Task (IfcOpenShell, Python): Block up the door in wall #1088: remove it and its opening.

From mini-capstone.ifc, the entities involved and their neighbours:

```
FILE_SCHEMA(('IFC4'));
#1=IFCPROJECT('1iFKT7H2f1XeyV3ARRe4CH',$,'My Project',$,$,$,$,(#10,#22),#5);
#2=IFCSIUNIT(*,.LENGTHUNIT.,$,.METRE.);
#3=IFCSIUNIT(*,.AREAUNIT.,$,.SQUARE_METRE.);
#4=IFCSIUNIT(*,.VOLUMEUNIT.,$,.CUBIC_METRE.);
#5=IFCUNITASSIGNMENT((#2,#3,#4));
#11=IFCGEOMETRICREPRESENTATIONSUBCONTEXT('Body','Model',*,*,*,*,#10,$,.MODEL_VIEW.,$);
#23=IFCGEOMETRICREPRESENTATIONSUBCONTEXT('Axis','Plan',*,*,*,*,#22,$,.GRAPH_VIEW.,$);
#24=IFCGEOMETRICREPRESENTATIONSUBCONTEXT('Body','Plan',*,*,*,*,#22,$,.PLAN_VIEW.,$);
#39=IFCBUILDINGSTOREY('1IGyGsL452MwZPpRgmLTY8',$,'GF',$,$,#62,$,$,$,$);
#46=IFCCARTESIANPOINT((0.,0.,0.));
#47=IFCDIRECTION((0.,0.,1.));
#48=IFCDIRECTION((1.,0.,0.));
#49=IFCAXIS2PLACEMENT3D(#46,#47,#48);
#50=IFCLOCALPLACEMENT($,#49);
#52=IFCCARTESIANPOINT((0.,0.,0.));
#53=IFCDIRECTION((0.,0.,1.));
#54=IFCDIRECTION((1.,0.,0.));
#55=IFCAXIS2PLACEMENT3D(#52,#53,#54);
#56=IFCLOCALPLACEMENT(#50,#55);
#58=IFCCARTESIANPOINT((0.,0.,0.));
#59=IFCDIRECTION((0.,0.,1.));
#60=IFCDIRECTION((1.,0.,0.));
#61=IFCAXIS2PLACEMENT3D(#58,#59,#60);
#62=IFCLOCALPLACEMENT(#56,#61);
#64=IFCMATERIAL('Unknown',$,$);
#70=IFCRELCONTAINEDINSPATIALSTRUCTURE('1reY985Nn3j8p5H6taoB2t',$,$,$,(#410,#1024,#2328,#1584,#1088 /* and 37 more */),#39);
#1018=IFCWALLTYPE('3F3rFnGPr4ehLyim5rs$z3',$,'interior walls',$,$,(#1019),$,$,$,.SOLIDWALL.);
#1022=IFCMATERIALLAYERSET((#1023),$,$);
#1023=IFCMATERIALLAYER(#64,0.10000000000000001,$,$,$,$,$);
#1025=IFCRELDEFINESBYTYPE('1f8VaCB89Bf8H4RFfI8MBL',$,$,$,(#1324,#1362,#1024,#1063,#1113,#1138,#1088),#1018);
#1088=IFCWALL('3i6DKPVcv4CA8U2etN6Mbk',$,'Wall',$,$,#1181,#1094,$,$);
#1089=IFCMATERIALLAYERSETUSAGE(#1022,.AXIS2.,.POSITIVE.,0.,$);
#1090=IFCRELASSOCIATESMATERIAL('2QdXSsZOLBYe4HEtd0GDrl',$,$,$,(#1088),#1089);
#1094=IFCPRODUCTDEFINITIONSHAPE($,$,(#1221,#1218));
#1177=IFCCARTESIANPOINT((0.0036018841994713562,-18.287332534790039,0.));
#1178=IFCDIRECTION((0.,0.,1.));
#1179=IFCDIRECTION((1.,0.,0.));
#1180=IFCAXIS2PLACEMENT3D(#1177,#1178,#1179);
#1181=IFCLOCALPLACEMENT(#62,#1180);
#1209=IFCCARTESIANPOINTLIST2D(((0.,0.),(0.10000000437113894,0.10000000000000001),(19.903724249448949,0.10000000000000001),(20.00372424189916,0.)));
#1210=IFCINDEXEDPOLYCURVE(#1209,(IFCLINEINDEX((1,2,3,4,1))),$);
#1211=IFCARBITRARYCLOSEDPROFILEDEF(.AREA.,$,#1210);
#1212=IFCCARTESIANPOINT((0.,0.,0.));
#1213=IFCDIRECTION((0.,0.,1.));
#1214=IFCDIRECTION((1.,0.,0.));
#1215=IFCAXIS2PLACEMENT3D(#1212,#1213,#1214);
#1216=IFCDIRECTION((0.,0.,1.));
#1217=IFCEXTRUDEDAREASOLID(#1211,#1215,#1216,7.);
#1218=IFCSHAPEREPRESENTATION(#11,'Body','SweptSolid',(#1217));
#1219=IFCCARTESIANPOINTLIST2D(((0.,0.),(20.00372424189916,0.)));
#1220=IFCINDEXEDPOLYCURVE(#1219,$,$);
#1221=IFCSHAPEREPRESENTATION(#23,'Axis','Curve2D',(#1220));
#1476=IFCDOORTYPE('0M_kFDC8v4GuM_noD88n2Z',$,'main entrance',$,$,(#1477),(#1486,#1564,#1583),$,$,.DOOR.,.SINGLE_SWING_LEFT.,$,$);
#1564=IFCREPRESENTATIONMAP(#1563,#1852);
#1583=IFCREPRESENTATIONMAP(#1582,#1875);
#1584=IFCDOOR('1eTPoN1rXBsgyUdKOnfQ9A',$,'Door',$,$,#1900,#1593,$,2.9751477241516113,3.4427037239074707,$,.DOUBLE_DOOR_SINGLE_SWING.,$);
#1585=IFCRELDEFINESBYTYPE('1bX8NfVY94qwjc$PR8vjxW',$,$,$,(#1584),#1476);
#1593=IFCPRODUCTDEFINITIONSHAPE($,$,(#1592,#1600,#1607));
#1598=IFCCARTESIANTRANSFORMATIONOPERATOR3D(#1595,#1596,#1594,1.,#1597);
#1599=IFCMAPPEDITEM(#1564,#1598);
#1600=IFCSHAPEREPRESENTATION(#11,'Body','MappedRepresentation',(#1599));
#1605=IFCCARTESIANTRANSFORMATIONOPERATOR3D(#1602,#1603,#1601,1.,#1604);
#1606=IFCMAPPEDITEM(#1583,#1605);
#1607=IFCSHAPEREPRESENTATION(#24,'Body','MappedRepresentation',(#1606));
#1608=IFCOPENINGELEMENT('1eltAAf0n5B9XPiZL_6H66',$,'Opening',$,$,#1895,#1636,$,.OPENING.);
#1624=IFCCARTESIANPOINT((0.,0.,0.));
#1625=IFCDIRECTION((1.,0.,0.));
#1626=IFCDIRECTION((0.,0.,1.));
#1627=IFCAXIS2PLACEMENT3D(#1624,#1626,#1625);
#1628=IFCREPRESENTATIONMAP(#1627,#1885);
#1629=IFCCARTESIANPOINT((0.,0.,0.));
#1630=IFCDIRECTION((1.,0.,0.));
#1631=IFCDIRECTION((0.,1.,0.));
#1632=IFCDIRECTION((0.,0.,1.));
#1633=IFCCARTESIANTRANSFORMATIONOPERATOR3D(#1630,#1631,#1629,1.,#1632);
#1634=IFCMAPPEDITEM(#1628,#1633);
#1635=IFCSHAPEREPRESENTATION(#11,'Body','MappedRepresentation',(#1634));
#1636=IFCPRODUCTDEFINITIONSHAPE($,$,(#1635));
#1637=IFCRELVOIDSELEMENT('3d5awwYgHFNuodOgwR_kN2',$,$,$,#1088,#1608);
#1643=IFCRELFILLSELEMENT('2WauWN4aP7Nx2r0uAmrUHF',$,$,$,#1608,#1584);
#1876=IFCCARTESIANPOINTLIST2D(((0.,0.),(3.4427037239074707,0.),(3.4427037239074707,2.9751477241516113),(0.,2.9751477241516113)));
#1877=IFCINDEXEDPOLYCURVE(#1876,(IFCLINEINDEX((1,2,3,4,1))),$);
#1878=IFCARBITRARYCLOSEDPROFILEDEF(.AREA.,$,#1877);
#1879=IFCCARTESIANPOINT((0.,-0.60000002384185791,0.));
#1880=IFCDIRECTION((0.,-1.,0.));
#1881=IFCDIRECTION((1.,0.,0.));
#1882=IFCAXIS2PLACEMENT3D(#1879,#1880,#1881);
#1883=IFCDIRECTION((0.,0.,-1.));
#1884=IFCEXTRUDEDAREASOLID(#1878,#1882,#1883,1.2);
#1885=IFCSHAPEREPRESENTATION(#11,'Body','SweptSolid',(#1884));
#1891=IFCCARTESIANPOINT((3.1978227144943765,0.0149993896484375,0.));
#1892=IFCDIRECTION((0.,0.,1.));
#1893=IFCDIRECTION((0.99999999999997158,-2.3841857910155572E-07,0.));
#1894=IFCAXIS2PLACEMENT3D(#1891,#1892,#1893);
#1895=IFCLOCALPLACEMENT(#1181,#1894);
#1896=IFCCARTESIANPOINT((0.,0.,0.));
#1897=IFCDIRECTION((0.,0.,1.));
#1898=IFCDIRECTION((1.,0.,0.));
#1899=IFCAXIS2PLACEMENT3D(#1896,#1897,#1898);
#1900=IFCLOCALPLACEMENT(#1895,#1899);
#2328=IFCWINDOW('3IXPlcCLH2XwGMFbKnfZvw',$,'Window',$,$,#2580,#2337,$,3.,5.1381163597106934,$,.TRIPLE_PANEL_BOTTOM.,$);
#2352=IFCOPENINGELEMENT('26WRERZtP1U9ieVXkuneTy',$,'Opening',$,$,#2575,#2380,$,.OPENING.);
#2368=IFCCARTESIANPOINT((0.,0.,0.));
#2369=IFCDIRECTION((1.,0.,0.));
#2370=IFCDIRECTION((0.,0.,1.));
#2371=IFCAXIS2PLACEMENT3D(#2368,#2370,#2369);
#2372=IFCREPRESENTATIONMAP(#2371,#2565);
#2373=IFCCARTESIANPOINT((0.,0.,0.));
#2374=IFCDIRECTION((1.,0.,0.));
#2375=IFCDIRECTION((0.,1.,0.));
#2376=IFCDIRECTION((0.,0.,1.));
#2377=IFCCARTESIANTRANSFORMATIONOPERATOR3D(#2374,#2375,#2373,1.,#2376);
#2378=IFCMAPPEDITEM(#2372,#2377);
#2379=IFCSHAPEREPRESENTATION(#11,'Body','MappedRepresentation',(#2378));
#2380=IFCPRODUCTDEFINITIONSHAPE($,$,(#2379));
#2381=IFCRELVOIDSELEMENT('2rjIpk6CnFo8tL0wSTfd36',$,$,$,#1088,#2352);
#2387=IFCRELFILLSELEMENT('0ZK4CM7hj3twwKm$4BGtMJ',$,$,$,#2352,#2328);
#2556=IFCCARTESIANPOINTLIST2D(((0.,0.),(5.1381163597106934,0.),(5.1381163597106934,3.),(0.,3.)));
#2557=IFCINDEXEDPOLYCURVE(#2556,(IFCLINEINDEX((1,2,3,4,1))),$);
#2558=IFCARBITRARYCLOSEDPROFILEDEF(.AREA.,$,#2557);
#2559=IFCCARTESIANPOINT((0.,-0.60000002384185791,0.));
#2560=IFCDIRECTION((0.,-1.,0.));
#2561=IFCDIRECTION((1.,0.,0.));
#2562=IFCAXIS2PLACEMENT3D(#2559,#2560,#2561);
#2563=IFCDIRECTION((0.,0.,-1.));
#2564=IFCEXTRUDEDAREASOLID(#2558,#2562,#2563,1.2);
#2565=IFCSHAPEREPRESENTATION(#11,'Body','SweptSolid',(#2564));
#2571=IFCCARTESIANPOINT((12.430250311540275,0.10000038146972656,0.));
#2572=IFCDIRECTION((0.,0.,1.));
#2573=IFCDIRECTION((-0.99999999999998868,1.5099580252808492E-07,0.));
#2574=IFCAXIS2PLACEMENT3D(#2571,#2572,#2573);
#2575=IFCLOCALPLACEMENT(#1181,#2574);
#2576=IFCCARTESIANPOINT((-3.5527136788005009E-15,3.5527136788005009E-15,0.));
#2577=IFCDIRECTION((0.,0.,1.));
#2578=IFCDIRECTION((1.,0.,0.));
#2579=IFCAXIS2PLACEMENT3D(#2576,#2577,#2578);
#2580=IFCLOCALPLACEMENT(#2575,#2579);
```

```python
import ifcopenshell
import ifcopenshell.api.feature
import ifcopenshell.api.root
import ifcopenshell.geom
import ifcopenshell.util.shape

model = ifcopenshell.open("mini-capstone.ifc")
settings = ifcopenshell.geom.settings()


def volume(element):
    """Net volume in cubic metres, openings subtracted."""
    shape = ifcopenshell.geom.create_shape(settings, element)
    return ifcopenshell.util.shape.get_volume(shape.geometry)


door = model.by_guid("1eTPoN1rXBsgyUdKOnfQ9A")
opening = door.FillsVoids[0].RelatingOpeningElement
wall = opening.VoidsElements[0].RelatingBuildingElement
before = volume(wall)

ifcopenshell.api.root.remove_product(model, product=door)
ifcopenshell.api.feature.remove_feature(model, feature=opening)

after = volume(wall)

print(f"wall volume {before:.3f} -> {after:.3f} m3")

model.write("mini-capstone-out.ifc")
```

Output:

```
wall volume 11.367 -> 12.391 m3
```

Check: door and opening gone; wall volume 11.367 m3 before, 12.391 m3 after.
